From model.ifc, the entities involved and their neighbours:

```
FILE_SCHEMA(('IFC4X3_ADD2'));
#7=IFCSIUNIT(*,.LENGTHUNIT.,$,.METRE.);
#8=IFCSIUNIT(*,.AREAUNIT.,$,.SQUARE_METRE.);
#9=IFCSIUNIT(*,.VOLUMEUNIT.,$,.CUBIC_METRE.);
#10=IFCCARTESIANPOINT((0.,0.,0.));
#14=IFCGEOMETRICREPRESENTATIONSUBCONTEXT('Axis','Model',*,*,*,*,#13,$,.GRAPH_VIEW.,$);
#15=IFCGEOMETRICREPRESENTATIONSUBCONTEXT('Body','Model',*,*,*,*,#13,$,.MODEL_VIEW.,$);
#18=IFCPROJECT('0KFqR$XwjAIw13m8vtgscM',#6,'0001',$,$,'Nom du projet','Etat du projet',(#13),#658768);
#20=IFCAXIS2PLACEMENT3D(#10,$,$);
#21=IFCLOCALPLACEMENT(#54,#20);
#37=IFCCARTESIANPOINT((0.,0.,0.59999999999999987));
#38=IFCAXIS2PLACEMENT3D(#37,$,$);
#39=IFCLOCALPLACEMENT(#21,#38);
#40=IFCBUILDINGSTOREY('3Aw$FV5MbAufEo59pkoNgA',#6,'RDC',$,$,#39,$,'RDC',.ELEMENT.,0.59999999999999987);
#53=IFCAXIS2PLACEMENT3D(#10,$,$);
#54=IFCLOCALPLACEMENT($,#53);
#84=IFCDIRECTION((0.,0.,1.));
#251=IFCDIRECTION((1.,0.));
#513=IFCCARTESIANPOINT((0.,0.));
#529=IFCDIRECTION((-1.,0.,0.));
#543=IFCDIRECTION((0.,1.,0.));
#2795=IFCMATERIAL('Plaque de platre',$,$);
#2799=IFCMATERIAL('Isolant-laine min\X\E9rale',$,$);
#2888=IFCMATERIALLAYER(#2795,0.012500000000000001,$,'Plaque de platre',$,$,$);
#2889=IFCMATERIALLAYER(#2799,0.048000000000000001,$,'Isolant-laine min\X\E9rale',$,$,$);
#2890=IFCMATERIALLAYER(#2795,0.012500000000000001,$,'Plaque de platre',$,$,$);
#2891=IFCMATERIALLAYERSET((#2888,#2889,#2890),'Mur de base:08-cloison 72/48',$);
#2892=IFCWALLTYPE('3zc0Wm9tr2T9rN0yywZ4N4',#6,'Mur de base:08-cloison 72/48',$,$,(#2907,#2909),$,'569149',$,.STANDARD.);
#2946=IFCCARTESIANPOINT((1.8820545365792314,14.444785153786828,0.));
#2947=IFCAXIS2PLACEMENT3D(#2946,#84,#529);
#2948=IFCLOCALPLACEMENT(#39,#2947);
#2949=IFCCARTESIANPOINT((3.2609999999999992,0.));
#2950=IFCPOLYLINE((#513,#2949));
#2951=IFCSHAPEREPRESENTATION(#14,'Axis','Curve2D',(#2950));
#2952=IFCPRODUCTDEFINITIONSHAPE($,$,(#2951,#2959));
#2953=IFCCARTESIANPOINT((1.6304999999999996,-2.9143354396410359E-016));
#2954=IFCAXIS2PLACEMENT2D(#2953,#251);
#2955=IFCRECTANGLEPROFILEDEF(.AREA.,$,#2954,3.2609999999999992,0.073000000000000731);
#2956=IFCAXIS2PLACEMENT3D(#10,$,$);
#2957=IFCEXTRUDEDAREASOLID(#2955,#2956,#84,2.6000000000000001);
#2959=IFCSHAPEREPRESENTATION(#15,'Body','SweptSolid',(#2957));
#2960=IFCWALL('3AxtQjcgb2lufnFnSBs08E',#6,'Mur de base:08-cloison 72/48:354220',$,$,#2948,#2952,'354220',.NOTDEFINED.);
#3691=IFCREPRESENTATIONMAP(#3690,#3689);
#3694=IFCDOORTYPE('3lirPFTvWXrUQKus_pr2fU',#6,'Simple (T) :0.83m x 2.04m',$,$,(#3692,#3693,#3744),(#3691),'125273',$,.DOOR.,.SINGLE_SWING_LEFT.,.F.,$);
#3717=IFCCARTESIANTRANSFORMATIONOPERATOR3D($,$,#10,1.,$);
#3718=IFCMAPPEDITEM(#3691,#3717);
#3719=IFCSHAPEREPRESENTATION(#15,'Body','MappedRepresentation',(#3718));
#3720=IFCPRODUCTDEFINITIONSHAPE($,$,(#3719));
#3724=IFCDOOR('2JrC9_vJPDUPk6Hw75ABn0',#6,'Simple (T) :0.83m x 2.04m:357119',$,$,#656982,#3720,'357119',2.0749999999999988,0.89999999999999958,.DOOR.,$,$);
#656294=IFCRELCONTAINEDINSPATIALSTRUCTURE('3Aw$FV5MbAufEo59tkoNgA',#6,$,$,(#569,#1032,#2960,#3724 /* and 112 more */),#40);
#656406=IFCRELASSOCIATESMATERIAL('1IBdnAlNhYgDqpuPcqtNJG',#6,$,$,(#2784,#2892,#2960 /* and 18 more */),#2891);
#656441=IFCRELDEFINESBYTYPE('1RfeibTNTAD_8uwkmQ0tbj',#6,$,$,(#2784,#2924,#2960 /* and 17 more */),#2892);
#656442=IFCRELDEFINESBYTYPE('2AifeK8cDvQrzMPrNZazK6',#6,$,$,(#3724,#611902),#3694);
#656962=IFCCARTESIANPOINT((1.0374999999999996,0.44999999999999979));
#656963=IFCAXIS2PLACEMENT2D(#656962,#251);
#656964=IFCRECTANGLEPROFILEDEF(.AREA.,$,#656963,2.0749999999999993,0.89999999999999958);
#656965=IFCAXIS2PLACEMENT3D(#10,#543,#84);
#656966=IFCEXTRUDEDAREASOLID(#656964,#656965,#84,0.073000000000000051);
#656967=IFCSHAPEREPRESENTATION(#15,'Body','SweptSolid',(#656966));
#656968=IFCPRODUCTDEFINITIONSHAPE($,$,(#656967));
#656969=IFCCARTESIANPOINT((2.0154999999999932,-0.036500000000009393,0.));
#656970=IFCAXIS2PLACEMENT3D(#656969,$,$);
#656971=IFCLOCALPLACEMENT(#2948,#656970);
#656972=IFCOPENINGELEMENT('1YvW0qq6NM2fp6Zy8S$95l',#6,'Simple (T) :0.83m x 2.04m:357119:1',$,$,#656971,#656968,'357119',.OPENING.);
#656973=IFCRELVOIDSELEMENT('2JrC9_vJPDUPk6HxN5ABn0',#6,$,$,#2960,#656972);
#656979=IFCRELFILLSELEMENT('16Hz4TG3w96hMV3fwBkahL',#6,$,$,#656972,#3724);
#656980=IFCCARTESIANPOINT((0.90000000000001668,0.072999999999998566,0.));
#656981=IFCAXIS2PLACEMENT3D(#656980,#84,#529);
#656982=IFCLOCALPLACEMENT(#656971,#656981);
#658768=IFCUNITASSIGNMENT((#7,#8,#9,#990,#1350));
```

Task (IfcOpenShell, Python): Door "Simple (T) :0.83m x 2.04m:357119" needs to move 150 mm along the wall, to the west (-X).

```python
import ifcopenshell
import ifcopenshell.api.geometry
import ifcopenshell.util.placement
import ifcopenshell.util.unit

model = ifcopenshell.open("model.ifc")
unit_scale = ifcopenshell.util.unit.calculate_unit_scale(model)

door = model.by_id(3724)
opening = door.FillsVoids[0].RelatingOpeningElement
wall = opening.VoidsElements[0].RelatingBuildingElement

wall_matrix = ifcopenshell.util.placement.get_local_placement(wall.ObjectPlacement)
shift = wall_matrix[:3, 0] * 0.15 / unit_scale
before = ifcopenshell.util.placement.get_local_placement(door.ObjectPlacement)[:3, 3].copy()

# The door is placed relative to its opening, so it follows when the opening moves.
matrix = ifcopenshell.util.placement.get_local_placement(opening.ObjectPlacement)
matrix[:3, 3] += shift
ifcopenshell.api.geometry.edit_object_placement(
    model, product=opening, matrix=matrix, is_si=False, should_transform_children=True
)

after = ifcopenshell.util.placement.get_local_placement(door.ObjectPlacement)[:3, 3]
print("door moved by", (after - before).round(3) + 0.0)

model.write("model_v2.ifc")
```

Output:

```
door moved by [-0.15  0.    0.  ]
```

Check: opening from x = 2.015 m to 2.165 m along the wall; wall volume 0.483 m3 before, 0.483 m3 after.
